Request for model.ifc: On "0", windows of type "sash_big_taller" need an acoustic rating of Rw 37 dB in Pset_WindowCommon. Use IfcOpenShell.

First a look at what the model holds.

```python
import ifcopenshell
import ifcopenshell.util.element

model = ifcopenshell.open("model.ifc")
print(model.schema)
storey = next(s for s in model.by_type("IfcBuildingStorey") if s.Name == "0")
windows = [e for e in ifcopenshell.util.element.get_decomposition(storey) if e.is_a("IfcWindow")]
seen = {}
for e in windows:
    element_type = ifcopenshell.util.element.get_type(e)
    key = (element_type.Name if element_type != e and element_type else None, ifcopenshell.util.element.get_pset(e, "Pset_WindowCommon", "AcousticRating"))
    seen[key] = seen.get(key, 0) + 1
for (name, value), count in sorted(seen.items(), key=str):
    print(count, "x", name, "|", value)
```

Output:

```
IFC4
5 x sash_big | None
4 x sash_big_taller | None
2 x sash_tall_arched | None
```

```python
import ifcopenshell
import ifcopenshell.api.pset
import ifcopenshell.util.element

model = ifcopenshell.open("model.ifc")

storey = next(s for s in model.by_type("IfcBuildingStorey") if s.Name == "0")
windows = [e for e in ifcopenshell.util.element.get_decomposition(storey) if e.is_a("IfcWindow")]

count = 0
for e in windows:
    element_type = ifcopenshell.util.element.get_type(e)
    if element_type in (None, e) or element_type.Name != "sash_big_taller":
        continue
    # add_pset returns the element's existing set when there is one.
    pset = ifcopenshell.api.pset.add_pset(model, product=e, name="Pset_WindowCommon")
    ifcopenshell.api.pset.edit_pset(model, pset=pset, properties={"AcousticRating": "Rw 37 dB"})
    count += 1

print(count, "windows updated")

model.write("model_v2.ifc")
```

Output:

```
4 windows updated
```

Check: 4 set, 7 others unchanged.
